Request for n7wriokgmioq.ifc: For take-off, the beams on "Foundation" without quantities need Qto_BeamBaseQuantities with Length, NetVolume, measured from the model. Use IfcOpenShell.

First a look at what the model holds.

```python
import ifcopenshell
import ifcopenshell.util.element
import ifcopenshell.util.unit

model = ifcopenshell.open("n7wriokgmioq.ifc")
print(model.schema)
for unit_type in ("LENGTHUNIT", "AREAUNIT", "VOLUMEUNIT"):
    print(unit_type, ifcopenshell.util.unit.calculate_unit_scale(model, unit_type))
storey = next(s for s in model.by_type("IfcBuildingStorey") if s.Name == "Foundation")
beams = [e for e in ifcopenshell.util.element.get_decomposition(storey) if e.is_a("IfcBeam")]
for e in sorted(beams, key=lambda e: e.id()):
    print(e.id(), e.is_a(), e.Name, list(ifcopenshell.util.element.get_psets(e, qtos_only=True)), sep=" | ")
```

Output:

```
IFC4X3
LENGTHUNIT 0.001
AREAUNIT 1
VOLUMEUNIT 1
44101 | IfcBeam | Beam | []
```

```python
import ifcopenshell
import ifcopenshell.api.pset
import ifcopenshell.geom
import ifcopenshell.util.element
import ifcopenshell.util.shape
import ifcopenshell.util.unit

model = ifcopenshell.open("n7wriokgmioq.ifc")
unit_scale = ifcopenshell.util.unit.calculate_unit_scale(model)
volume_scale = ifcopenshell.util.unit.calculate_unit_scale(model, "VOLUMEUNIT")
settings = ifcopenshell.geom.settings()

storey = next(s for s in model.by_type("IfcBuildingStorey") if s.Name == "Foundation")
beams = [e for e in ifcopenshell.util.element.get_decomposition(storey) if e.is_a("IfcBeam")]

for e in sorted(beams, key=lambda e: e.id()):
    if ifcopenshell.util.element.get_psets(e, qtos_only=True, should_inherit=False):
        continue
    # Geometry comes back in metres, in the element's own axes.
    shape = ifcopenshell.geom.create_shape(settings, e)
    values = {
        "Length": ifcopenshell.util.shape.get_max_xyz(shape.geometry) / unit_scale,
        "NetVolume": ifcopenshell.util.shape.get_volume(shape.geometry) / volume_scale,
    }
    qto = ifcopenshell.api.pset.add_qto(model, product=e, name="Qto_BeamBaseQuantities")
    ifcopenshell.api.pset.edit_qto(model, qto=qto, properties=values)
    print(e.id(), {k: round(v, 3) for k, v in values.items()})

model.write("n7wriokgmioq_edited.ifc")
```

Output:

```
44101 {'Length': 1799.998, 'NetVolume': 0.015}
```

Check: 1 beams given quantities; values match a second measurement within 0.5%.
